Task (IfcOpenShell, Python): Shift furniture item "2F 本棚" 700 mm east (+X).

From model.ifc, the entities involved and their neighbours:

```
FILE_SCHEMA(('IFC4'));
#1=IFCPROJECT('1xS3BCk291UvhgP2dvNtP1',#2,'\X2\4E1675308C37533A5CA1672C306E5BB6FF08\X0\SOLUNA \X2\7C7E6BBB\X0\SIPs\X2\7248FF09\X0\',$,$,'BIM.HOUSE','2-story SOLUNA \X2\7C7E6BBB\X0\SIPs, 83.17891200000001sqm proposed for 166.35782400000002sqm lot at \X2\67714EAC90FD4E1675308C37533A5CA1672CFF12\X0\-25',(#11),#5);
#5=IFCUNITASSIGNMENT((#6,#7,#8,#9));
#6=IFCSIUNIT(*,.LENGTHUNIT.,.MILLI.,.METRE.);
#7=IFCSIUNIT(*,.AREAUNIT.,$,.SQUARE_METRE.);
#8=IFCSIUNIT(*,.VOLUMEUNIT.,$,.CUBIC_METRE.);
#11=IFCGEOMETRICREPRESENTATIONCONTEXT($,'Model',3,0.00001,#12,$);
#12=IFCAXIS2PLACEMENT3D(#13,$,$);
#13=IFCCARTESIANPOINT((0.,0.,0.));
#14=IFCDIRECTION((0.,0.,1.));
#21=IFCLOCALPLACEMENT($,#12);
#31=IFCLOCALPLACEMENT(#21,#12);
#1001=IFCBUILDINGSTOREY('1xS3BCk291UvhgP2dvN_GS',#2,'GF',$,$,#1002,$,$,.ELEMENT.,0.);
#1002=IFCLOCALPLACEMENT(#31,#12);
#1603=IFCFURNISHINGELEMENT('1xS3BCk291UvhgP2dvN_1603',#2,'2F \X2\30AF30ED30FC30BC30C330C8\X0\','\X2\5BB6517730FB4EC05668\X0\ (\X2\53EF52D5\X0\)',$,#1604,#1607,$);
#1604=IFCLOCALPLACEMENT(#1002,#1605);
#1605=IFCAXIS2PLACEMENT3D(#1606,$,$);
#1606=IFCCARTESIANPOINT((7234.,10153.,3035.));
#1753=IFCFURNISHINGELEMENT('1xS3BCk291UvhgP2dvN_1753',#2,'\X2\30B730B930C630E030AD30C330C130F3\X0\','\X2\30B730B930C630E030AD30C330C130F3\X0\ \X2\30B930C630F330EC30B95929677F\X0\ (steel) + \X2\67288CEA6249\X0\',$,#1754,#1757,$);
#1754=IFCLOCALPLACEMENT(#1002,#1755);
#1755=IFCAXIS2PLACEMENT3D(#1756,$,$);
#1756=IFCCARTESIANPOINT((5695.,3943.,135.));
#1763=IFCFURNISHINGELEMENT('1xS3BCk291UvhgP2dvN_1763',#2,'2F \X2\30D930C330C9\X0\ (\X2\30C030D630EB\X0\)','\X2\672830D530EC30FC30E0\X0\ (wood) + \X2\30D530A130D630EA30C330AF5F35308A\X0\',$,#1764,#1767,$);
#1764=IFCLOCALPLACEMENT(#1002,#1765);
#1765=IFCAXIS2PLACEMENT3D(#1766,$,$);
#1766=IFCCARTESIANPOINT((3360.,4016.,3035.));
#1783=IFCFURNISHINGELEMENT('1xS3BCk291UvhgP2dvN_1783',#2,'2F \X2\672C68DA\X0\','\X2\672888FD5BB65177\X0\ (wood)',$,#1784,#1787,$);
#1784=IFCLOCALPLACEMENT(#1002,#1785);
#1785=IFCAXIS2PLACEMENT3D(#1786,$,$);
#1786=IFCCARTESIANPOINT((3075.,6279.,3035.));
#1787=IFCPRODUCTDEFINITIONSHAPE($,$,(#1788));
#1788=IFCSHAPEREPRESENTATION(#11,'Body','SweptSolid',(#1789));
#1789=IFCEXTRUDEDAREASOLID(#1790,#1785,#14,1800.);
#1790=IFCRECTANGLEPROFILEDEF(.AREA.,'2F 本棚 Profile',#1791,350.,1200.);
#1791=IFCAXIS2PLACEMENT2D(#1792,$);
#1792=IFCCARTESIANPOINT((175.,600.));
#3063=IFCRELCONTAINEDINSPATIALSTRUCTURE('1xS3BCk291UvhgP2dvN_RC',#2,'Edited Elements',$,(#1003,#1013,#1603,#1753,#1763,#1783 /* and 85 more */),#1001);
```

```python
import ifcopenshell
import ifcopenshell.api.geometry
import ifcopenshell.util.placement
import ifcopenshell.util.unit

model = ifcopenshell.open("model.ifc")
unit_scale = ifcopenshell.util.unit.calculate_unit_scale(model)

item = model.by_guid("1xS3BCk291UvhgP2dvN_1783")
matrix = ifcopenshell.util.placement.get_local_placement(item.ObjectPlacement)
matrix[0, 3] += 0.7 / unit_scale
ifcopenshell.api.geometry.edit_object_placement(model, product=item, matrix=matrix, is_si=False)

print(ifcopenshell.util.placement.get_local_placement(item.ObjectPlacement).round(3) + 0.0)

model.write("model_updated.ifc")
```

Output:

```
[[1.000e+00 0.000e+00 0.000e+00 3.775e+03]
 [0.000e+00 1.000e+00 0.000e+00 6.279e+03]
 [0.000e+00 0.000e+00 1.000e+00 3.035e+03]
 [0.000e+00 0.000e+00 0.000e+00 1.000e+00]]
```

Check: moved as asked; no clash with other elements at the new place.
